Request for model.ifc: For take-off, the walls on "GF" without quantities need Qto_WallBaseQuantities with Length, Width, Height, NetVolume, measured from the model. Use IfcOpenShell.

First a look at what the model holds.

```python
import ifcopenshell
import ifcopenshell.util.element
import ifcopenshell.util.unit

model = ifcopenshell.open("model.ifc")
print(model.schema)
for unit_type in ("LENGTHUNIT", "AREAUNIT", "VOLUMEUNIT"):
    print(unit_type, ifcopenshell.util.unit.calculate_unit_scale(model, unit_type))
storey = next(s for s in model.by_type("IfcBuildingStorey") if s.Name == "GF")
walls = [e for e in ifcopenshell.util.element.get_decomposition(storey) if e.is_a("IfcWall")]
for e in sorted(walls, key=lambda e: e.id()):
    print(e.id(), e.is_a(), e.Name, list(ifcopenshell.util.element.get_psets(e, qtos_only=True)), sep=" | ")
```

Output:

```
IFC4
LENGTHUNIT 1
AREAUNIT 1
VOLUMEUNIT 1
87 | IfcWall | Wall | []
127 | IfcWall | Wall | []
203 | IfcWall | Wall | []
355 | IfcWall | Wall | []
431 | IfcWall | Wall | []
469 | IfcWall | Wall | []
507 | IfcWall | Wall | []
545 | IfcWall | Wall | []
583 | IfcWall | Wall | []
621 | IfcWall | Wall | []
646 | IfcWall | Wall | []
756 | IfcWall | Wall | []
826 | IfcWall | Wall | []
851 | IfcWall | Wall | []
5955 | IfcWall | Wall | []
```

```python
import ifcopenshell
import ifcopenshell.api.pset
import ifcopenshell.geom
import ifcopenshell.util.element
import ifcopenshell.util.shape
import ifcopenshell.util.unit

model = ifcopenshell.open("model.ifc")
unit_scale = ifcopenshell.util.unit.calculate_unit_scale(model)
volume_scale = ifcopenshell.util.unit.calculate_unit_scale(model, "VOLUMEUNIT")
settings = ifcopenshell.geom.settings()

storey = next(s for s in model.by_type("IfcBuildingStorey") if s.Name == "GF")
walls = [e for e in ifcopenshell.util.element.get_decomposition(storey) if e.is_a("IfcWall")]

for e in sorted(walls, key=lambda e: e.id()):
    if ifcopenshell.util.element.get_psets(e, qtos_only=True, should_inherit=False):
        continue
    # Geometry comes back in metres, in the element's own axes.
    shape = ifcopenshell.geom.create_shape(settings, e)
    values = {
        "Length": ifcopenshell.util.shape.get_x(shape.geometry) / unit_scale,
        "Width": ifcopenshell.util.shape.get_y(shape.geometry) / unit_scale,
        "Height": ifcopenshell.util.shape.get_z(shape.geometry) / unit_scale,
        "NetVolume": ifcopenshell.util.shape.get_volume(shape.geometry) / volume_scale,
    }
    qto = ifcopenshell.api.pset.add_qto(model, product=e, name="Qto_WallBaseQuantities")
    ifcopenshell.api.pset.edit_qto(model, qto=qto, properties=values)
    print(e.id(), {k: round(v, 3) for k, v in values.items()})

model.write("model-out.ifc")
```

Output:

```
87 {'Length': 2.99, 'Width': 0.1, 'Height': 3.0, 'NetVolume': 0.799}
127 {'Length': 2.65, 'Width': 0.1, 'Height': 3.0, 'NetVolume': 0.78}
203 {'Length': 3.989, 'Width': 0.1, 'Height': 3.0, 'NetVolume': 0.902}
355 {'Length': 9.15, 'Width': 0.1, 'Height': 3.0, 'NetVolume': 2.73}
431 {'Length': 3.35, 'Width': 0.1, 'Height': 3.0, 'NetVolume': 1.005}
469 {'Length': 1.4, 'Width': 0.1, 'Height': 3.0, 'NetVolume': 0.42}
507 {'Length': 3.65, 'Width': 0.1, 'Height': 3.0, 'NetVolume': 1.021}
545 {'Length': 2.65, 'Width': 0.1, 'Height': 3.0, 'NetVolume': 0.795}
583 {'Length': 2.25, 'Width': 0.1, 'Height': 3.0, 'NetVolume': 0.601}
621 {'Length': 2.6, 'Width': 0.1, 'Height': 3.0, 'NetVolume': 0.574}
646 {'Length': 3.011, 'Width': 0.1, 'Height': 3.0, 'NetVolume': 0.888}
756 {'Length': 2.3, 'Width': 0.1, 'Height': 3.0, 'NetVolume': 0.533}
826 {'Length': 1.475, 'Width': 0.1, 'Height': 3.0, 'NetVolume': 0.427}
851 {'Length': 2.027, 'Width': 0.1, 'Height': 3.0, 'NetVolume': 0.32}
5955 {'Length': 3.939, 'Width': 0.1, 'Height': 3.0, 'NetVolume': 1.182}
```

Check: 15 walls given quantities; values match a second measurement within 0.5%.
